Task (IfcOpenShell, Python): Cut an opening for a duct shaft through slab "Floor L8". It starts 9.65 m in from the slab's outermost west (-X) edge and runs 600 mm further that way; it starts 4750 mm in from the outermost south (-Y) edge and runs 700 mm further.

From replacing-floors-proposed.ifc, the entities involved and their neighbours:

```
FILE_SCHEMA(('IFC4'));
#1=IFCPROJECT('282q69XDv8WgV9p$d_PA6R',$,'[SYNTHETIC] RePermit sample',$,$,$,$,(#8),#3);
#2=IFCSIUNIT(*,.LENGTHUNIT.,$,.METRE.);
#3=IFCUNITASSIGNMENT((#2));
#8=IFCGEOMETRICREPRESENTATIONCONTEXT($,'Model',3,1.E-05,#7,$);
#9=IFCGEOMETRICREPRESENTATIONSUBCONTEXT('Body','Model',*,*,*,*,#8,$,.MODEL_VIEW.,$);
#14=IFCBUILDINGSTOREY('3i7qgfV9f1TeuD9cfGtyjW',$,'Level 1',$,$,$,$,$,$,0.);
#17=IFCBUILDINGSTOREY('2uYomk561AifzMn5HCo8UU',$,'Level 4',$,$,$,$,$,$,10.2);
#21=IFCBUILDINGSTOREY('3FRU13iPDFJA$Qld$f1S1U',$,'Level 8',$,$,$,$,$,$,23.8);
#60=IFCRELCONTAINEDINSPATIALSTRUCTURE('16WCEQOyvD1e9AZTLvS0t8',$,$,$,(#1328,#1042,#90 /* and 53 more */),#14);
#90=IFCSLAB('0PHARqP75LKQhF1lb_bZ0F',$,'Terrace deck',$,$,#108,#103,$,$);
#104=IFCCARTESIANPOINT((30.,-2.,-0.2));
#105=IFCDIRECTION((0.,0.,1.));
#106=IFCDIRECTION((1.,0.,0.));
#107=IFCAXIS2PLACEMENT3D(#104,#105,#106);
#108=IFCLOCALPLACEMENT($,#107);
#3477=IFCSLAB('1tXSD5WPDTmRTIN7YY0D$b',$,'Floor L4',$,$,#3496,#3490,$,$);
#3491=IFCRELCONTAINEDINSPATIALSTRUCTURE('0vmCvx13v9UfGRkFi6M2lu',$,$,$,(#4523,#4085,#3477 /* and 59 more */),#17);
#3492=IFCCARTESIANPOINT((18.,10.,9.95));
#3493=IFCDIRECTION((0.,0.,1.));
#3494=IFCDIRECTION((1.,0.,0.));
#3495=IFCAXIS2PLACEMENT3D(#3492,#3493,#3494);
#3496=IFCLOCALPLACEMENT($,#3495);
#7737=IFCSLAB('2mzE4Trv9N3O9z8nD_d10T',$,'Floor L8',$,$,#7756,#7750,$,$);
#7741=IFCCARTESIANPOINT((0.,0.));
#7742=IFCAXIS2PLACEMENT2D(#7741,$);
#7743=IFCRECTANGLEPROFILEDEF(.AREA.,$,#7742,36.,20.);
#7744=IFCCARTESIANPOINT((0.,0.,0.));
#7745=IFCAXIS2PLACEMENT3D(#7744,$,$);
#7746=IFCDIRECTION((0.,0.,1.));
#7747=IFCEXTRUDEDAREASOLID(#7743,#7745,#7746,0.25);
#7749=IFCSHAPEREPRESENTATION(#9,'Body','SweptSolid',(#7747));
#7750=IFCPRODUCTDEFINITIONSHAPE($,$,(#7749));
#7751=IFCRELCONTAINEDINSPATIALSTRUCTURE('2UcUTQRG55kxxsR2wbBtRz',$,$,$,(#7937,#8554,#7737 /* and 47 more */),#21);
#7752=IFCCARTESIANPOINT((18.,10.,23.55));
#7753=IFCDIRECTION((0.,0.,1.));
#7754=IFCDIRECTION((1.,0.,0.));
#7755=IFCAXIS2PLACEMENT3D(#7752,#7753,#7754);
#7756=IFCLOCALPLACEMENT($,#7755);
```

```python
import numpy as np
import ifcopenshell
import ifcopenshell.api.feature
import ifcopenshell.api.geometry
import ifcopenshell.api.root
import ifcopenshell.geom
import ifcopenshell.util.placement
import ifcopenshell.util.representation
import ifcopenshell.util.shape
import ifcopenshell.util.unit

model = ifcopenshell.open("replacing-floors-proposed.ifc")
unit_scale = ifcopenshell.util.unit.calculate_unit_scale(model)
settings = ifcopenshell.geom.settings()


def volume(element):
    """Net volume in cubic metres, openings subtracted."""
    shape = ifcopenshell.geom.create_shape(settings, element)
    return ifcopenshell.util.shape.get_volume(shape.geometry)


slab = model.by_guid("2mzE4Trv9N3O9z8nD_d10T")
before = volume(slab)

# Extent in the slab's own axes, in metres. The edges named are its -X and -Y sides.
slab_shape = ifcopenshell.geom.create_shape(settings, slab)
vertices = ifcopenshell.util.shape.get_vertices(slab_shape.geometry)
x_min, y_min, bottom = vertices.min(axis=0)
top = vertices[:, 2].max()

opening = ifcopenshell.api.root.create_entity(model, ifc_class="IfcOpeningElement", name="Duct shaft opening", predefined_type="OPENING")
context = ifcopenshell.util.representation.get_context(model, "Model", "Body", "MODEL_VIEW")
width, depth = 0.6, 0.7
outline = [(0.0, 0.0), (width, 0.0), (width, depth), (0.0, depth), (0.0, 0.0)]
# Overshoot both faces by 50 mm so the cut is clean.
shape = ifcopenshell.api.geometry.add_slab_representation(
    model, context=context, depth=top - bottom + 0.1, polyline=outline
)
ifcopenshell.api.geometry.assign_representation(model, product=opening, representation=shape)

matrix = ifcopenshell.util.placement.get_local_placement(slab.ObjectPlacement)
matrix[:, 3] = matrix @ np.append(np.array([x_min + 9.65, y_min + 4.75, bottom - 0.05]) / unit_scale, 1.0)
ifcopenshell.api.geometry.edit_object_placement(model, product=opening, matrix=matrix, is_si=False)
ifcopenshell.api.feature.add_feature(model, feature=opening, element=slab)

after = volume(slab)

print(f"slab volume {before:.3f} -> {after:.3f} m3")

model.write("replacing-floors-proposed_rev.ifc")
```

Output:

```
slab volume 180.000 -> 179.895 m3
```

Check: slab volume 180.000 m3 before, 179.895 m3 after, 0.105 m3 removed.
